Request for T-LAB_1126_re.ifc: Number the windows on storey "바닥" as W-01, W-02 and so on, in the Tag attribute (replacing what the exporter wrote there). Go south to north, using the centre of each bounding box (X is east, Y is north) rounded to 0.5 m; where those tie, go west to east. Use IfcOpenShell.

First a look at what the model holds.

```python
import ifcopenshell
import ifcopenshell.util.element
import ifcopenshell.util.placement

model = ifcopenshell.open("T-LAB_1126_re.ifc")
print(model.schema)
storey = next(s for s in model.by_type("IfcBuildingStorey") if s.Name == "바닥")
windows = [e for e in ifcopenshell.util.element.get_decomposition(storey) if e.is_a("IfcWindow")]
for e in sorted(windows, key=lambda e: e.id()):
    origin = ifcopenshell.util.placement.get_local_placement(e.ObjectPlacement)[:3, 3]
    print(e.id(), e.Tag, e.Name, origin.round(2) + 0.0, sep=" | ")
```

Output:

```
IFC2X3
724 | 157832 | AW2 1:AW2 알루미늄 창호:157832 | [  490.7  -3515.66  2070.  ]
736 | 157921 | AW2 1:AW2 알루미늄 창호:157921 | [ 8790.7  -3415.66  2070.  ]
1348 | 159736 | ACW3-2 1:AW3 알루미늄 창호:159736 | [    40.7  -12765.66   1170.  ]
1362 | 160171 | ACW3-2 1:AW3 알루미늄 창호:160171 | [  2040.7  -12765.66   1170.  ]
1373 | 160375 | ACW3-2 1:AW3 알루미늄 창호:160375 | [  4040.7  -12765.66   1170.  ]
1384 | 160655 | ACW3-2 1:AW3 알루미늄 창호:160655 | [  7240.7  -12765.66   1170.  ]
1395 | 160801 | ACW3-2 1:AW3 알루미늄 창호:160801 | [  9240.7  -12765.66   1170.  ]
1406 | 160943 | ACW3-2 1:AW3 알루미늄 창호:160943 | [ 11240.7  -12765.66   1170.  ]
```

```python
import ifcopenshell
import ifcopenshell.geom
import ifcopenshell.util.element
import ifcopenshell.util.shape

model = ifcopenshell.open("T-LAB_1126_re.ifc")
settings = ifcopenshell.geom.settings()
settings.set("use-world-coords", True)


def centre(element):
    shape = ifcopenshell.geom.create_shape(settings, element)
    return ifcopenshell.util.shape.get_bbox_centroid(shape.geometry)


storey = next(s for s in model.by_type("IfcBuildingStorey") if s.Name == "바닥")
windows = [e for e in ifcopenshell.util.element.get_decomposition(storey) if e.is_a("IfcWindow")]

# Insertion points can sit at a corner or the storey origin, so sort by the geometry (in metres).
centres = {e: centre(e) for e in windows}
windows.sort(key=lambda e: (round(centres[e][1] / 0.5), centres[e][0]))

for i, e in enumerate(windows, start=1):
    number = f"W-{i:02d}"
    e.Tag = number
    print(e.id(), number)

model.write("T-LAB_1126_re_rev.ifc")
```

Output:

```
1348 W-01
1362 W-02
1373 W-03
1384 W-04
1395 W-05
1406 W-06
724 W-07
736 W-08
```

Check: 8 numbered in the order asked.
